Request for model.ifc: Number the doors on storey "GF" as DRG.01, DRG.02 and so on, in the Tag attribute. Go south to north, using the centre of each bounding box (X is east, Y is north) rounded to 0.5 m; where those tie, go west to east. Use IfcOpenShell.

First a look at what the model holds.

```python
import ifcopenshell
import ifcopenshell.util.element
import ifcopenshell.util.placement

model = ifcopenshell.open("model.ifc")
print(model.schema)
storey = next(s for s in model.by_type("IfcBuildingStorey") if s.Name == "GF")
doors = [e for e in ifcopenshell.util.element.get_decomposition(storey) if e.is_a("IfcDoor")]
for e in sorted(doors, key=lambda e: e.id()):
    origin = ifcopenshell.util.placement.get_local_placement(e.ObjectPlacement)[:3, 3]
    print(e.id(), e.Tag, e.Name, origin.round(2) + 0.0, sep=" | ")
```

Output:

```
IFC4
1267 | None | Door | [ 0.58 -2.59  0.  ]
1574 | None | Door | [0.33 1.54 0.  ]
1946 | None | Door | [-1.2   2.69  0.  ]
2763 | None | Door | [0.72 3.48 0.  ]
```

```python
import ifcopenshell
import ifcopenshell.geom
import ifcopenshell.util.element
import ifcopenshell.util.shape

model = ifcopenshell.open("model.ifc")
settings = ifcopenshell.geom.settings()
settings.set("use-world-coords", True)


def centre(element):
    shape = ifcopenshell.geom.create_shape(settings, element)
    return ifcopenshell.util.shape.get_bbox_centroid(shape.geometry)


storey = next(s for s in model.by_type("IfcBuildingStorey") if s.Name == "GF")
doors = [e for e in ifcopenshell.util.element.get_decomposition(storey) if e.is_a("IfcDoor")]

# Insertion points can sit at a corner or the storey origin, so sort by the geometry (in metres).
centres = {e: centre(e) for e in doors}
doors.sort(key=lambda e: (round(centres[e][1] / 0.5), centres[e][0]))

for i, e in enumerate(doors, start=1):
    number = f"DRG.{i:02d}"
    e.Tag = number
    print(e.id(), number)

model.write("model_rev.ifc")
```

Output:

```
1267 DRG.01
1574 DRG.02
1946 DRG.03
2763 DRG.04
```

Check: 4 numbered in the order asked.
